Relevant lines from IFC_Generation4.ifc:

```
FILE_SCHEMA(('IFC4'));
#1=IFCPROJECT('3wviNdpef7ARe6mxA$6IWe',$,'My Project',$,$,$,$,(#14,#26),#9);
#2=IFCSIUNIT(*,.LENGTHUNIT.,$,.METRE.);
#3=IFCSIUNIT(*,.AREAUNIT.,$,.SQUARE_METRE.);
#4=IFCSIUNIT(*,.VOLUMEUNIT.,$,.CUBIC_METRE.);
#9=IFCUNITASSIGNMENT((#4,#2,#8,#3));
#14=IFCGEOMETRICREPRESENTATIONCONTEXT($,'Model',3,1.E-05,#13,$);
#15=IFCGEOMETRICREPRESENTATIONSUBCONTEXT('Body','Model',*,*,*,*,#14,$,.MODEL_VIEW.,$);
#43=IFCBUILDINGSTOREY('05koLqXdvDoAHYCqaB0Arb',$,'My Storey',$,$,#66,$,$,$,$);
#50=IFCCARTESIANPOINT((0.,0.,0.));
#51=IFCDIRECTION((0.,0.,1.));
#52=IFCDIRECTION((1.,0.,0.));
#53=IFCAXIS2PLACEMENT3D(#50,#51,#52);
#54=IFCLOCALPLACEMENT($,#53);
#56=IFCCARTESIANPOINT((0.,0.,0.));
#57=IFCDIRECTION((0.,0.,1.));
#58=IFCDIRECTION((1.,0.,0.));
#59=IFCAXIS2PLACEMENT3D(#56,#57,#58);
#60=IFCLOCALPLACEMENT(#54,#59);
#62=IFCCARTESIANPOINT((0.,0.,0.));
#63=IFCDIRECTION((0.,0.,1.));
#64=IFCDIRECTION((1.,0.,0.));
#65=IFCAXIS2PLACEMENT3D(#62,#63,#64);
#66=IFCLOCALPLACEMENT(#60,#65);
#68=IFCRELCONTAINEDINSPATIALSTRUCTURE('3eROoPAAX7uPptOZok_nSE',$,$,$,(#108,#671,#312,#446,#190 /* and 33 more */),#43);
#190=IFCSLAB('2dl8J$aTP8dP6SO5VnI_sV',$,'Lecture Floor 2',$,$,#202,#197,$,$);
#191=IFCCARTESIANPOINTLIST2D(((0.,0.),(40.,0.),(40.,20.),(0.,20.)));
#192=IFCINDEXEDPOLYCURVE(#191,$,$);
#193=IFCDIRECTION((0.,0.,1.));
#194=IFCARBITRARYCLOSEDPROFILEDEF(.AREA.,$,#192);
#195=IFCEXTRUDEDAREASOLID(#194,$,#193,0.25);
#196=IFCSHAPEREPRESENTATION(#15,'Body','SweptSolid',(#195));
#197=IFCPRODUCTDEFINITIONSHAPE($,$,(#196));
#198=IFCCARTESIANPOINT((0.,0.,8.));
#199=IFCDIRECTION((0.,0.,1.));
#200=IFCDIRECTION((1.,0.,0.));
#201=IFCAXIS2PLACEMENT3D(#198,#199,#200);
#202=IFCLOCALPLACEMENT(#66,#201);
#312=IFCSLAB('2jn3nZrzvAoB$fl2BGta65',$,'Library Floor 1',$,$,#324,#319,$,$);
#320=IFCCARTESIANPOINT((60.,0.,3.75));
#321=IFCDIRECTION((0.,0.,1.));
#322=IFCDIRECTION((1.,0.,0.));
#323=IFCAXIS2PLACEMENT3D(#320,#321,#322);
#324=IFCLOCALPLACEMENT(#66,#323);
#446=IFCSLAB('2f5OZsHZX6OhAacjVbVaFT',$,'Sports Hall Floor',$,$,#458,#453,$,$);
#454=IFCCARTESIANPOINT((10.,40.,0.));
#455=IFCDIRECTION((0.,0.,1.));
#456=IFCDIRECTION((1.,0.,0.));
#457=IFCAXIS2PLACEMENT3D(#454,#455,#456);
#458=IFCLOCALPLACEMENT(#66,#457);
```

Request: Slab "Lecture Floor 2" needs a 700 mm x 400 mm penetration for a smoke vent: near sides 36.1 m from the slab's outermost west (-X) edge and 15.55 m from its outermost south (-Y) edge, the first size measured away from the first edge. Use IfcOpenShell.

```python
import numpy as np
import ifcopenshell
import ifcopenshell.api.feature
import ifcopenshell.api.geometry
import ifcopenshell.api.root
import ifcopenshell.geom
import ifcopenshell.util.placement
import ifcopenshell.util.representation
import ifcopenshell.util.shape
import ifcopenshell.util.unit

model = ifcopenshell.open("IFC_Generation4.ifc")
unit_scale = ifcopenshell.util.unit.calculate_unit_scale(model)
settings = ifcopenshell.geom.settings()


def volume(element):
    """Net volume in cubic metres, openings subtracted."""
    shape = ifcopenshell.geom.create_shape(settings, element)
    return ifcopenshell.util.shape.get_volume(shape.geometry)


slab = model.by_guid("2dl8J$aTP8dP6SO5VnI_sV")
before = volume(slab)

# Extent in the slab's own axes, in metres. The edges named are its -X and -Y sides.
slab_shape = ifcopenshell.geom.create_shape(settings, slab)
vertices = ifcopenshell.util.shape.get_vertices(slab_shape.geometry)
x_min, y_min, bottom = vertices.min(axis=0)
top = vertices[:, 2].max()

opening = ifcopenshell.api.root.create_entity(model, ifc_class="IfcOpeningElement", name="Smoke vent opening", predefined_type="OPENING")
context = ifcopenshell.util.representation.get_context(model, "Model", "Body", "MODEL_VIEW")
width, depth = 0.7, 0.4
outline = [(0.0, 0.0), (width, 0.0), (width, depth), (0.0, depth), (0.0, 0.0)]
# Overshoot both faces by 50 mm so the cut is clean.
shape = ifcopenshell.api.geometry.add_slab_representation(
    model, context=context, depth=top - bottom + 0.1, polyline=outline
)
ifcopenshell.api.geometry.assign_representation(model, product=opening, representation=shape)

matrix = ifcopenshell.util.placement.get_local_placement(slab.ObjectPlacement)
matrix[:, 3] = matrix @ np.append(np.array([x_min + 36.1, y_min + 15.55, bottom - 0.05]) / unit_scale, 1.0)
ifcopenshell.api.geometry.edit_object_placement(model, product=opening, matrix=matrix, is_si=False)
ifcopenshell.api.feature.add_feature(model, feature=opening, element=slab)

after = volume(slab)

print(f"slab volume {before:.3f} -> {after:.3f} m3")

model.write("IFC_Generation4-out.ifc")
```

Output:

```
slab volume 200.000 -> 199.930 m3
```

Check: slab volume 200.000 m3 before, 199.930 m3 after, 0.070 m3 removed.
